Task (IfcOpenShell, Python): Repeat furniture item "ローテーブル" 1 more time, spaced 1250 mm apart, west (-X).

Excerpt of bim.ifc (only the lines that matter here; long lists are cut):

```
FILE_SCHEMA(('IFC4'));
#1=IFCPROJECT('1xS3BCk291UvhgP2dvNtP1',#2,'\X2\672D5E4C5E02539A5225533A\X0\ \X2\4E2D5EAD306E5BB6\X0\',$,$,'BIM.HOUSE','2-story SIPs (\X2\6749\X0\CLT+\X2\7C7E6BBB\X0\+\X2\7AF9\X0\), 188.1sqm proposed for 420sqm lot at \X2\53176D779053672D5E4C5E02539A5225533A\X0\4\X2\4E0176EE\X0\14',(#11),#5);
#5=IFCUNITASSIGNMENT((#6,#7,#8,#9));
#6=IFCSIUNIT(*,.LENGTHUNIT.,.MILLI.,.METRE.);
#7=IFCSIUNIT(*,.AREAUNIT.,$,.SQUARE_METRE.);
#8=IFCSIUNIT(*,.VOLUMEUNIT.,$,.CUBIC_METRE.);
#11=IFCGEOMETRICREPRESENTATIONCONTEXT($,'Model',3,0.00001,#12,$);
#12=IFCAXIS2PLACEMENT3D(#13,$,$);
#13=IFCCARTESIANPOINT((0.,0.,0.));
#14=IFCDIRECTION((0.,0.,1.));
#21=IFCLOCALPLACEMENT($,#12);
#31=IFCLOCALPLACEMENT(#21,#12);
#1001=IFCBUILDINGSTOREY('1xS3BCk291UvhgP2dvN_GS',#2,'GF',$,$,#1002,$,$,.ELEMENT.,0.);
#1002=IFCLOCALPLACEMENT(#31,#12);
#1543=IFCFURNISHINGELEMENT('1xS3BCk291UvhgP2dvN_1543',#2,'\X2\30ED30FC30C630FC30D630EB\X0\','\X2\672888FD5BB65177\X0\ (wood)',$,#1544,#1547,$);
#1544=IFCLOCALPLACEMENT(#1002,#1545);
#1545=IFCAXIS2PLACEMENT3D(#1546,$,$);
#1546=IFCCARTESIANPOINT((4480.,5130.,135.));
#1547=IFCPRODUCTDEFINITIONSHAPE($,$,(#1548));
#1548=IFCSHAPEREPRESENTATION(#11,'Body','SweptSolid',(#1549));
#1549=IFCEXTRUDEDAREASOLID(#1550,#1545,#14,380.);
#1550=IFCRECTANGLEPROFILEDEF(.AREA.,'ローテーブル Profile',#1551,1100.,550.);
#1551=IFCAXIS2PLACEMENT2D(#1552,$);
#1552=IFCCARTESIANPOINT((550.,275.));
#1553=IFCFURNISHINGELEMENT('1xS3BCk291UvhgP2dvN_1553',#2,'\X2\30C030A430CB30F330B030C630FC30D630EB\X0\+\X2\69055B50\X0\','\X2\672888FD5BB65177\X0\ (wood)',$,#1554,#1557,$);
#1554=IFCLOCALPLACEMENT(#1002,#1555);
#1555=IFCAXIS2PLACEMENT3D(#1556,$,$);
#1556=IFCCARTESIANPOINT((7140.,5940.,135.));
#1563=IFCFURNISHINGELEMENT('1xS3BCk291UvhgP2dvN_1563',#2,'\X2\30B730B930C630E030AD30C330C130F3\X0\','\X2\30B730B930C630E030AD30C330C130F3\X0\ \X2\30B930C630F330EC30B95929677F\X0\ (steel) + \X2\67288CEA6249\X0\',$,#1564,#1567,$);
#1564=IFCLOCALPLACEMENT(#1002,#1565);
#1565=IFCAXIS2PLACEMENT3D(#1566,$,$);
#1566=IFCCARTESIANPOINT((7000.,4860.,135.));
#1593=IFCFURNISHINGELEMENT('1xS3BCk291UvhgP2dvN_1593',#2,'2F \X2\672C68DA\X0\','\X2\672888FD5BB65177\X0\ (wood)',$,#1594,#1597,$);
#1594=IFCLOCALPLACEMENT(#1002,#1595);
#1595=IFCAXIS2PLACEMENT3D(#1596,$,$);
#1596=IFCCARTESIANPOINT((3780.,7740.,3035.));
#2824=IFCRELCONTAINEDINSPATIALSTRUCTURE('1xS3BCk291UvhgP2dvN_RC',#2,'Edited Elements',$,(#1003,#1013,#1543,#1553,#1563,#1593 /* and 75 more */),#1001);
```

```python
import numpy as np
import ifcopenshell
import ifcopenshell.api.geometry
import ifcopenshell.api.root
import ifcopenshell.util.element
import ifcopenshell.util.placement
import ifcopenshell.util.unit

model = ifcopenshell.open("bim.ifc")
unit_scale = ifcopenshell.util.unit.calculate_unit_scale(model)


def reuse_history(source, copy):
    """copy_class also copies each property set's owner history, people and application; keep the originals."""
    for rel in copy.IsDefinedBy:
        if rel.is_a("IfcRelDefinesByProperties") and (history := rel.RelatingPropertyDefinition.OwnerHistory):
            rel.RelatingPropertyDefinition.OwnerHistory = source.OwnerHistory
            ifcopenshell.util.element.remove_deep2(model, history)


source = model.by_guid("1xS3BCk291UvhgP2dvN_1543")
base = ifcopenshell.util.placement.get_local_placement(source.ObjectPlacement)
step = np.array([-1.0, 0.0, 0.0]) * 1.25 / unit_scale

for i in range(1, 2):
    copy = ifcopenshell.api.root.copy_class(model, product=source)
    copy.Representation = ifcopenshell.util.element.copy_deep(
        model, source.Representation, exclude=["IfcGeometricRepresentationContext", "IfcRepresentationMap"]
    )
    reuse_history(source, copy)
    matrix = base.copy()
    matrix[:3, 3] += i * step
    print("added at", matrix[:3, 3].round(3) + 0.0)
    ifcopenshell.api.geometry.edit_object_placement(model, product=copy, matrix=matrix, is_si=False)

model.write("bim_updated.ifc")
```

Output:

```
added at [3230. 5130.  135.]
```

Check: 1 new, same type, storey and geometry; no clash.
